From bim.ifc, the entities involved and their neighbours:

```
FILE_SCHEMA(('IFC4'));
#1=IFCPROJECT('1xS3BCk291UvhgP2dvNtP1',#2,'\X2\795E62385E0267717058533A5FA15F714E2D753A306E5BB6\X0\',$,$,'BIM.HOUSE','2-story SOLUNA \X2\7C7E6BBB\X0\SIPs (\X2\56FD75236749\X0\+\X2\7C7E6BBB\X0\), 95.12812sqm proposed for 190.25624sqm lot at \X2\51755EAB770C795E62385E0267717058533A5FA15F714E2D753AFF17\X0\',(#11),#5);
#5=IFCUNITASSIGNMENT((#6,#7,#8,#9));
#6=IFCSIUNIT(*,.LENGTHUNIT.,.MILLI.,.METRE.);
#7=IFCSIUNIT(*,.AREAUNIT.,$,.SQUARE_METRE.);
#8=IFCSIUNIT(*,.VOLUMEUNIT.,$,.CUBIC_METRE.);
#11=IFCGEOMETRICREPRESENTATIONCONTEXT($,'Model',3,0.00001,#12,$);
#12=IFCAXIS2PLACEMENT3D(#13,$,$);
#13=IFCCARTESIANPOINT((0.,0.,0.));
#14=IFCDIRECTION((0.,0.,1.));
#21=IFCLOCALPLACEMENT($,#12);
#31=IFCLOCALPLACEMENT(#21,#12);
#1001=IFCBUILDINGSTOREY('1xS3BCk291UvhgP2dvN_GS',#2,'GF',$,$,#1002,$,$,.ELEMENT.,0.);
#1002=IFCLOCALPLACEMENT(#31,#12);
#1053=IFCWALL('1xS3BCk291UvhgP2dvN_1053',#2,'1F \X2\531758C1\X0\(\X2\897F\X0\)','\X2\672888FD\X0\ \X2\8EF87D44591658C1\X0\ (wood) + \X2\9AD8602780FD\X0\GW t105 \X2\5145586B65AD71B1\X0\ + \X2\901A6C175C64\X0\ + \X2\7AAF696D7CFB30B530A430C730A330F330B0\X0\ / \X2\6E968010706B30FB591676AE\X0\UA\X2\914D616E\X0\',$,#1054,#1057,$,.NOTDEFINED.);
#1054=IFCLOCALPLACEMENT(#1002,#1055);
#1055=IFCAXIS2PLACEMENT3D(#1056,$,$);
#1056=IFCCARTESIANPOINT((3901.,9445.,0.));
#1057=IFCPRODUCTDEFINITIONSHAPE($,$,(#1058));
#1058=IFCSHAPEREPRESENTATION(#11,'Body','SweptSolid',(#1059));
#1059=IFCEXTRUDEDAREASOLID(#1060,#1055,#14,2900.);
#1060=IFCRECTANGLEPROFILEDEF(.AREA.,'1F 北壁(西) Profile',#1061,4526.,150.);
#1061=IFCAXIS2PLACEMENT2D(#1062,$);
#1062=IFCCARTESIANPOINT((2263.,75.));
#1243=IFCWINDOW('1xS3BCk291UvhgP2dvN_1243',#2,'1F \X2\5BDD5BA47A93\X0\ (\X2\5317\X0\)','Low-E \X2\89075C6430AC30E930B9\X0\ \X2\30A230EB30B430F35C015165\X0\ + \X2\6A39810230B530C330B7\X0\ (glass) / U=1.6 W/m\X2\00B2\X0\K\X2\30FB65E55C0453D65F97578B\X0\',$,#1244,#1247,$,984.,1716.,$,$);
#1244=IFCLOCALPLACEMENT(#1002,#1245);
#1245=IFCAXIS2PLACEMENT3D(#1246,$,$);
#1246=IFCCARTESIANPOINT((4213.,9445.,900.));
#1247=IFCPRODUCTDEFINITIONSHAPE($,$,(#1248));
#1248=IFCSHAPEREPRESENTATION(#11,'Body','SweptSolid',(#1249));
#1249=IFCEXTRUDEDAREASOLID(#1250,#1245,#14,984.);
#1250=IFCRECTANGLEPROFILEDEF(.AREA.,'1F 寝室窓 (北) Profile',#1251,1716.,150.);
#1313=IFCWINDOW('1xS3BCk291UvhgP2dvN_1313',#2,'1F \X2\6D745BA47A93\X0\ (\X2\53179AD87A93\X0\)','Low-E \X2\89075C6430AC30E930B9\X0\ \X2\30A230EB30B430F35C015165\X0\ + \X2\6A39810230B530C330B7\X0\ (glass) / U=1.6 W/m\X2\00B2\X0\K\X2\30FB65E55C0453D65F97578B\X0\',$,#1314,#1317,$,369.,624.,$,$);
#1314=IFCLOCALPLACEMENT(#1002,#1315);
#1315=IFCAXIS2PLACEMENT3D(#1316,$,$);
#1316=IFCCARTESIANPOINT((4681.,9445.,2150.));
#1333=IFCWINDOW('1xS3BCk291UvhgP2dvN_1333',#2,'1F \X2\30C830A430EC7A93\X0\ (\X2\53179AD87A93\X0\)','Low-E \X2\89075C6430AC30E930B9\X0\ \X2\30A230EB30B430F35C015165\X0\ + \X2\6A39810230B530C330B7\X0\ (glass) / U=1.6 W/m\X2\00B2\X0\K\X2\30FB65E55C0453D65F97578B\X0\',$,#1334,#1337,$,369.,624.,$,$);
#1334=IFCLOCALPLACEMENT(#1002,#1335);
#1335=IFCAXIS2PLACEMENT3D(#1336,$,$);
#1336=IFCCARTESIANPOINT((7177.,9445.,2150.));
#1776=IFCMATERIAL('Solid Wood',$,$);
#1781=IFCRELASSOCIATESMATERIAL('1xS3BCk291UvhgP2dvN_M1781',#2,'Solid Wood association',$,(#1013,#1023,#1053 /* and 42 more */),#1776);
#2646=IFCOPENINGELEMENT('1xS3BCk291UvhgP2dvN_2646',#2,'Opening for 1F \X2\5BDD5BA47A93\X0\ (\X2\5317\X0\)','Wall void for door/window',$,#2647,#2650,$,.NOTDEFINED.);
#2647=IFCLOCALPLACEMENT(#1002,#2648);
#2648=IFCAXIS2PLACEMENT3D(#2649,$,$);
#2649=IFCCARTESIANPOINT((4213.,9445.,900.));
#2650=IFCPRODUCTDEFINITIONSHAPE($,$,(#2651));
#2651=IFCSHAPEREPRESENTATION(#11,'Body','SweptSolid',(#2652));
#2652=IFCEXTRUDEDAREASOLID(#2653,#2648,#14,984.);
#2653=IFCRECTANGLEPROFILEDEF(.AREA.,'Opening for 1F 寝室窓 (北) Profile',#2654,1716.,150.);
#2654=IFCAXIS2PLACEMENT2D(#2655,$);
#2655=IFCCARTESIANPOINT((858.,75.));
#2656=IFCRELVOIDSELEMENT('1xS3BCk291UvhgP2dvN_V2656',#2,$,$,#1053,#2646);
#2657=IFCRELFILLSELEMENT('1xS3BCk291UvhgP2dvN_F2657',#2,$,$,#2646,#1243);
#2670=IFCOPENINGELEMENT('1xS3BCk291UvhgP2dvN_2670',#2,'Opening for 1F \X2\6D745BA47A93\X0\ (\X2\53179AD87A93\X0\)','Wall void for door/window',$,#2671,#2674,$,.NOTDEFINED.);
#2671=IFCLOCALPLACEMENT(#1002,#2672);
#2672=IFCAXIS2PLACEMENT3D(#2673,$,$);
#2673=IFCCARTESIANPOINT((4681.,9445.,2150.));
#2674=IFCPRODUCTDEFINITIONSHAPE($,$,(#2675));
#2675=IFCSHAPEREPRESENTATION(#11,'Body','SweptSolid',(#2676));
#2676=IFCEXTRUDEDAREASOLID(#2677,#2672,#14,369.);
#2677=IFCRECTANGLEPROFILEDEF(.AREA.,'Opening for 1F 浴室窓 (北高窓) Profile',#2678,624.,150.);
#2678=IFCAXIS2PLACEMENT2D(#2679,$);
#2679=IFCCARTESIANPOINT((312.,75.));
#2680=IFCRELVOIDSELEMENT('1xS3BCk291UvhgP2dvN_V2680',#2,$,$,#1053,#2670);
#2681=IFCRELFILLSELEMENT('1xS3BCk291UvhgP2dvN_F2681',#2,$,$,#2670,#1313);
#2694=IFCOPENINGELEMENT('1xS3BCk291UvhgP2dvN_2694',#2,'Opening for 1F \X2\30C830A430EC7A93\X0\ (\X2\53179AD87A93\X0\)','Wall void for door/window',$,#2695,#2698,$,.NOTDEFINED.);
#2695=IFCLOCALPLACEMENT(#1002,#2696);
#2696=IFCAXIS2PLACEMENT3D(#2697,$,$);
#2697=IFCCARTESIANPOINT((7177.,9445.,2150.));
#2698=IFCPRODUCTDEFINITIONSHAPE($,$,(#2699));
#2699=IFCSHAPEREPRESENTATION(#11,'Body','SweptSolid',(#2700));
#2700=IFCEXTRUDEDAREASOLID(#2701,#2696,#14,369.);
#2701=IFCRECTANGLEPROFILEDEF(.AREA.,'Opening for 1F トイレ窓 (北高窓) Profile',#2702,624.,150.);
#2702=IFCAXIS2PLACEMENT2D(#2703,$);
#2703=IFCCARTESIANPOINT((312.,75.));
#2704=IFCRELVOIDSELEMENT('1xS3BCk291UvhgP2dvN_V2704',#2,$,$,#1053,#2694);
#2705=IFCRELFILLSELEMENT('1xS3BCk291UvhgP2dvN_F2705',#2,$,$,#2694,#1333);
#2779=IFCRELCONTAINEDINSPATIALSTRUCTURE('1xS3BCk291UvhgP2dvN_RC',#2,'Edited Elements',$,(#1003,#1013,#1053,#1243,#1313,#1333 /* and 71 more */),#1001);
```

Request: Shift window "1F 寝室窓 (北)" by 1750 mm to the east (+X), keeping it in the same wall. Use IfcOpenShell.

```python
import ifcopenshell
import ifcopenshell.api.geometry
import ifcopenshell.util.placement
import ifcopenshell.util.unit

model = ifcopenshell.open("bim.ifc")
unit_scale = ifcopenshell.util.unit.calculate_unit_scale(model)

window = model.by_guid("1xS3BCk291UvhgP2dvN_1243")
opening = window.FillsVoids[0].RelatingOpeningElement
wall = opening.VoidsElements[0].RelatingBuildingElement

wall_matrix = ifcopenshell.util.placement.get_local_placement(wall.ObjectPlacement)
shift = wall_matrix[:3, 0] * 1.75 / unit_scale
before = ifcopenshell.util.placement.get_local_placement(window.ObjectPlacement)[:3, 3].copy()

# The window is not placed relative to its opening, so move both.
for product in (opening, window):
    matrix = ifcopenshell.util.placement.get_local_placement(product.ObjectPlacement)
    matrix[:3, 3] += shift
    ifcopenshell.api.geometry.edit_object_placement(model, product=product, matrix=matrix, is_si=False)

after = ifcopenshell.util.placement.get_local_placement(window.ObjectPlacement)[:3, 3]
print("window moved by", (after - before).round(3) + 0.0)

model.write("bim_v2.ifc")
```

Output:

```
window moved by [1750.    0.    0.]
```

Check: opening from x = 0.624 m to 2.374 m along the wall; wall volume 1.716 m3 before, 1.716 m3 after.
